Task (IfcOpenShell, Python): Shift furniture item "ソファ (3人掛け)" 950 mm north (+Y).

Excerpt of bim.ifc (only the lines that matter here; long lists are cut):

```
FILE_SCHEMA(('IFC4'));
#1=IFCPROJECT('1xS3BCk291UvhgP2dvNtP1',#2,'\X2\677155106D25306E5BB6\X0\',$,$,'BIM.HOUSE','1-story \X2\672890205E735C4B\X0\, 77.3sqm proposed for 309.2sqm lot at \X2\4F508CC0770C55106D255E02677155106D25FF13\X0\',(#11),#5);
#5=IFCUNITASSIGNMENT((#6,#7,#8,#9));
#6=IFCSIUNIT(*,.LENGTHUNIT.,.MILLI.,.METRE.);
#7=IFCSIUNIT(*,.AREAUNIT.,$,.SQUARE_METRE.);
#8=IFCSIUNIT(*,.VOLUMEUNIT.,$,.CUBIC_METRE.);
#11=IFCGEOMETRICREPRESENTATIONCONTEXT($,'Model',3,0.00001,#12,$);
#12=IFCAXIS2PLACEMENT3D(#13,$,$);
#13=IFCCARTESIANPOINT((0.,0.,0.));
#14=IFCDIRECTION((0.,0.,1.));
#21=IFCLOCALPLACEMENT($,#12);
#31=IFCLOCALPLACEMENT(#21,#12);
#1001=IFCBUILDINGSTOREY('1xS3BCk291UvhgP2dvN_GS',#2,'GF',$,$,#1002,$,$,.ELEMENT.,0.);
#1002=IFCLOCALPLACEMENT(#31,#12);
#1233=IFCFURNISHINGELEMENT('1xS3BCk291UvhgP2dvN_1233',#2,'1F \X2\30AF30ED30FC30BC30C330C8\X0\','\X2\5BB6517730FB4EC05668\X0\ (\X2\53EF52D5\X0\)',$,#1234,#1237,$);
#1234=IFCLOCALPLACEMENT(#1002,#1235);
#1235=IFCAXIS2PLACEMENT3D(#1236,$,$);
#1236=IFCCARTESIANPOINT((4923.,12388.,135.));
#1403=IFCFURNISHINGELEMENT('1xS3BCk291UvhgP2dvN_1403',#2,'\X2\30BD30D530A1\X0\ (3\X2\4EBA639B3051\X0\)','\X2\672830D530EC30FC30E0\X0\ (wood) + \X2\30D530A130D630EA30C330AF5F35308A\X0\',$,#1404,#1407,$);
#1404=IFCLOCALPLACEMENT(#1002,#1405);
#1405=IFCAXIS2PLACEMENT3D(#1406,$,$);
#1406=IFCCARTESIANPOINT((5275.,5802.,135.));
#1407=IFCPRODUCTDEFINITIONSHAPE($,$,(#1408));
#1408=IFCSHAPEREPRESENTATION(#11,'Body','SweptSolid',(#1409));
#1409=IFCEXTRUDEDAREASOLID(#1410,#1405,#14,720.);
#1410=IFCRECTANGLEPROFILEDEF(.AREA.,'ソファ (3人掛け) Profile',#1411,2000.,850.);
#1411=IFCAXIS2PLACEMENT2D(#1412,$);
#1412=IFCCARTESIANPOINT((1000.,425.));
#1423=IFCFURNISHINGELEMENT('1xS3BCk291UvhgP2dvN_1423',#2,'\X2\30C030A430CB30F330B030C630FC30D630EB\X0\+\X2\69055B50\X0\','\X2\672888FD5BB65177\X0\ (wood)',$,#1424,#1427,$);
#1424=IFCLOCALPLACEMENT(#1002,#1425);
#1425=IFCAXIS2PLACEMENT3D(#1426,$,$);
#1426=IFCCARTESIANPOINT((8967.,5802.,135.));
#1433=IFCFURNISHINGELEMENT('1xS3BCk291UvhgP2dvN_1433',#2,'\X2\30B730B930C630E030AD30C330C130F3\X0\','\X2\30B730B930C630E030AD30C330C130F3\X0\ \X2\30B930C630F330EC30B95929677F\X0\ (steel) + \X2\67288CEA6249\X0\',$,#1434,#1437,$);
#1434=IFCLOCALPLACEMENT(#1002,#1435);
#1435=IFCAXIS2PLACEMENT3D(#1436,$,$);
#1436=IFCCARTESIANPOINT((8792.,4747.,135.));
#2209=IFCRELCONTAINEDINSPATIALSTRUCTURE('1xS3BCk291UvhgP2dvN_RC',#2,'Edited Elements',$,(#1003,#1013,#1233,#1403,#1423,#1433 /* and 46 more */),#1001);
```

```python
import ifcopenshell
import ifcopenshell.api.geometry
import ifcopenshell.util.placement
import ifcopenshell.util.unit

model = ifcopenshell.open("bim.ifc")
unit_scale = ifcopenshell.util.unit.calculate_unit_scale(model)

item = model.by_id(1403)
matrix = ifcopenshell.util.placement.get_local_placement(item.ObjectPlacement)
matrix[1, 3] += 0.95 / unit_scale
ifcopenshell.api.geometry.edit_object_placement(model, product=item, matrix=matrix, is_si=False)

print(ifcopenshell.util.placement.get_local_placement(item.ObjectPlacement).round(3) + 0.0)

model.write("bim-out.ifc")
```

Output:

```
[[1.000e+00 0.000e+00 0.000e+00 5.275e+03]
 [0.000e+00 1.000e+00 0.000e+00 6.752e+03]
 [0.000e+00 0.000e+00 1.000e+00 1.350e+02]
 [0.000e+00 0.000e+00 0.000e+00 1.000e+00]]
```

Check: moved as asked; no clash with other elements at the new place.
